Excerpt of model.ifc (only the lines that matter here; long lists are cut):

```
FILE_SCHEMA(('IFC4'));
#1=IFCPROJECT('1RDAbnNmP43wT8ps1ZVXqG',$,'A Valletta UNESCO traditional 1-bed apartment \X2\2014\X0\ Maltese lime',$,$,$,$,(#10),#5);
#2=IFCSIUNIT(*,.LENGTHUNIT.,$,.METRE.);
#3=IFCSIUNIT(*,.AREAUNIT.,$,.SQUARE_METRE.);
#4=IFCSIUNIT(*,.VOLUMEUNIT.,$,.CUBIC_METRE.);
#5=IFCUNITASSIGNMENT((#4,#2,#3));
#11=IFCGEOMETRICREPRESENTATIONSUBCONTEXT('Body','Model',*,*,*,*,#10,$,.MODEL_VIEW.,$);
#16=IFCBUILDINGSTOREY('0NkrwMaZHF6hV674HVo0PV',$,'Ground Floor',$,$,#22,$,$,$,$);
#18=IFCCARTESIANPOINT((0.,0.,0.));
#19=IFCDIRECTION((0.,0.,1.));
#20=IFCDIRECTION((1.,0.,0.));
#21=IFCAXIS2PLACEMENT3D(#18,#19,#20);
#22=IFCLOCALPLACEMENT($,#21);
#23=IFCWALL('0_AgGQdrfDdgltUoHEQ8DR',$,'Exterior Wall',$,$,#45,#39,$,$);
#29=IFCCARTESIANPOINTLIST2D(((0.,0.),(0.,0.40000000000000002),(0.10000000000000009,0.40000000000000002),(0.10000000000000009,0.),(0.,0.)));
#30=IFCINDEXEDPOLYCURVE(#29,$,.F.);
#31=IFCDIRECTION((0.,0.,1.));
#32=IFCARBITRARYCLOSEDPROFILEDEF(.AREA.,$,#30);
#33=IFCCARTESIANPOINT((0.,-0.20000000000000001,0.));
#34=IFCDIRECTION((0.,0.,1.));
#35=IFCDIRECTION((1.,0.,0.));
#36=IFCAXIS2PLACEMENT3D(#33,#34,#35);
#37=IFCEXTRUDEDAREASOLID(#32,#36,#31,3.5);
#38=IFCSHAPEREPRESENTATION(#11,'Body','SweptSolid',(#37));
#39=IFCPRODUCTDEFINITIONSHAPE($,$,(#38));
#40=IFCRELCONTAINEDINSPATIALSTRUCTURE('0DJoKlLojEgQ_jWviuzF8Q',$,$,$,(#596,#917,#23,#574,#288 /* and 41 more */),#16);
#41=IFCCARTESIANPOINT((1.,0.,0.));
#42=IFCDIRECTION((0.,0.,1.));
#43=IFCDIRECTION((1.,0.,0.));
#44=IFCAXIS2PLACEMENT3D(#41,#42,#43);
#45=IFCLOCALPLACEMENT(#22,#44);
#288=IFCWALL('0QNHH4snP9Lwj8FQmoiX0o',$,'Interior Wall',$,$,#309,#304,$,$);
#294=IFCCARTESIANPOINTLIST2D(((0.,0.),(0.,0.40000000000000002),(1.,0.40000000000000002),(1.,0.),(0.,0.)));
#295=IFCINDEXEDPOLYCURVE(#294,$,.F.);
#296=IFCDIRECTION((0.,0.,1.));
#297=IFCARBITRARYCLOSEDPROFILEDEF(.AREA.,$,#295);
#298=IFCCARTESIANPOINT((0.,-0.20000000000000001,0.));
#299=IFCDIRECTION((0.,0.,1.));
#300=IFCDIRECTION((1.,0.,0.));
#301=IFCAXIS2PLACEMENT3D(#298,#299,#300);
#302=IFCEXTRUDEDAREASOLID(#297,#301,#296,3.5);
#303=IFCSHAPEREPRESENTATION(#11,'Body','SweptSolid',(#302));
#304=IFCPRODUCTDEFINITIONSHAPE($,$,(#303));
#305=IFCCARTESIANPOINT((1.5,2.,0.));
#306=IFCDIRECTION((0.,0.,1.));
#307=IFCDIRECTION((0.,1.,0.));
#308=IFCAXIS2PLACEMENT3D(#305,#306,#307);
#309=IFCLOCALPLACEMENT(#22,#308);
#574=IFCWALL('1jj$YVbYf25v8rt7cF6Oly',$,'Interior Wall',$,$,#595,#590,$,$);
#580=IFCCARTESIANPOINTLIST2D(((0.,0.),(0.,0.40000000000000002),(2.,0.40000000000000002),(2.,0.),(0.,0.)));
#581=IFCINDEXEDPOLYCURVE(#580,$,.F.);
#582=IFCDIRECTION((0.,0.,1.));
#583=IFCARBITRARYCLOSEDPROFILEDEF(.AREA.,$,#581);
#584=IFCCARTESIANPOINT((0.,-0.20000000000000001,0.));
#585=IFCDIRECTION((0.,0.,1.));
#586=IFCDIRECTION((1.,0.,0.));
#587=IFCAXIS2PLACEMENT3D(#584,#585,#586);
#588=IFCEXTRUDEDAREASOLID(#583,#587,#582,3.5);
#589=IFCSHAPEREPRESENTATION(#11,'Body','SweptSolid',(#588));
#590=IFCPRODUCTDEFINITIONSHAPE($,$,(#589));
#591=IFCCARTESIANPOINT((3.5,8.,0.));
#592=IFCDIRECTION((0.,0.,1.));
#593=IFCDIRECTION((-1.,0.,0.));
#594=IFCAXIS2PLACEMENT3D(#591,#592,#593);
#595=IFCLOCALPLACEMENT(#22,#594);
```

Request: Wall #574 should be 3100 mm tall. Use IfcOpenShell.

```python
import ifcopenshell
import ifcopenshell.geom
import ifcopenshell.util.representation
import ifcopenshell.util.shape

model = ifcopenshell.open("model.ifc")
settings = ifcopenshell.geom.settings()


def volume(element):
    """Net volume in cubic metres, openings subtracted."""
    shape = ifcopenshell.geom.create_shape(settings, element)
    return ifcopenshell.util.shape.get_volume(shape.geometry)


wall = model.by_guid("1jj$YVbYf25v8rt7cF6Oly")
before = volume(wall)

body = ifcopenshell.util.representation.get_representation(wall, "Model", "Body")
solid = body.Items[0]
old_height = solid.Depth
solid.Depth = 3.1
after = volume(wall)

print(f"height {old_height:g} -> {solid.Depth:g}, volume {before:.3f} -> {after:.3f} m3")

model.write("model-out.ifc")
```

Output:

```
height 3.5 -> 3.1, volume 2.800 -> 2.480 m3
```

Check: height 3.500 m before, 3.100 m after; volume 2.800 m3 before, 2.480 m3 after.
